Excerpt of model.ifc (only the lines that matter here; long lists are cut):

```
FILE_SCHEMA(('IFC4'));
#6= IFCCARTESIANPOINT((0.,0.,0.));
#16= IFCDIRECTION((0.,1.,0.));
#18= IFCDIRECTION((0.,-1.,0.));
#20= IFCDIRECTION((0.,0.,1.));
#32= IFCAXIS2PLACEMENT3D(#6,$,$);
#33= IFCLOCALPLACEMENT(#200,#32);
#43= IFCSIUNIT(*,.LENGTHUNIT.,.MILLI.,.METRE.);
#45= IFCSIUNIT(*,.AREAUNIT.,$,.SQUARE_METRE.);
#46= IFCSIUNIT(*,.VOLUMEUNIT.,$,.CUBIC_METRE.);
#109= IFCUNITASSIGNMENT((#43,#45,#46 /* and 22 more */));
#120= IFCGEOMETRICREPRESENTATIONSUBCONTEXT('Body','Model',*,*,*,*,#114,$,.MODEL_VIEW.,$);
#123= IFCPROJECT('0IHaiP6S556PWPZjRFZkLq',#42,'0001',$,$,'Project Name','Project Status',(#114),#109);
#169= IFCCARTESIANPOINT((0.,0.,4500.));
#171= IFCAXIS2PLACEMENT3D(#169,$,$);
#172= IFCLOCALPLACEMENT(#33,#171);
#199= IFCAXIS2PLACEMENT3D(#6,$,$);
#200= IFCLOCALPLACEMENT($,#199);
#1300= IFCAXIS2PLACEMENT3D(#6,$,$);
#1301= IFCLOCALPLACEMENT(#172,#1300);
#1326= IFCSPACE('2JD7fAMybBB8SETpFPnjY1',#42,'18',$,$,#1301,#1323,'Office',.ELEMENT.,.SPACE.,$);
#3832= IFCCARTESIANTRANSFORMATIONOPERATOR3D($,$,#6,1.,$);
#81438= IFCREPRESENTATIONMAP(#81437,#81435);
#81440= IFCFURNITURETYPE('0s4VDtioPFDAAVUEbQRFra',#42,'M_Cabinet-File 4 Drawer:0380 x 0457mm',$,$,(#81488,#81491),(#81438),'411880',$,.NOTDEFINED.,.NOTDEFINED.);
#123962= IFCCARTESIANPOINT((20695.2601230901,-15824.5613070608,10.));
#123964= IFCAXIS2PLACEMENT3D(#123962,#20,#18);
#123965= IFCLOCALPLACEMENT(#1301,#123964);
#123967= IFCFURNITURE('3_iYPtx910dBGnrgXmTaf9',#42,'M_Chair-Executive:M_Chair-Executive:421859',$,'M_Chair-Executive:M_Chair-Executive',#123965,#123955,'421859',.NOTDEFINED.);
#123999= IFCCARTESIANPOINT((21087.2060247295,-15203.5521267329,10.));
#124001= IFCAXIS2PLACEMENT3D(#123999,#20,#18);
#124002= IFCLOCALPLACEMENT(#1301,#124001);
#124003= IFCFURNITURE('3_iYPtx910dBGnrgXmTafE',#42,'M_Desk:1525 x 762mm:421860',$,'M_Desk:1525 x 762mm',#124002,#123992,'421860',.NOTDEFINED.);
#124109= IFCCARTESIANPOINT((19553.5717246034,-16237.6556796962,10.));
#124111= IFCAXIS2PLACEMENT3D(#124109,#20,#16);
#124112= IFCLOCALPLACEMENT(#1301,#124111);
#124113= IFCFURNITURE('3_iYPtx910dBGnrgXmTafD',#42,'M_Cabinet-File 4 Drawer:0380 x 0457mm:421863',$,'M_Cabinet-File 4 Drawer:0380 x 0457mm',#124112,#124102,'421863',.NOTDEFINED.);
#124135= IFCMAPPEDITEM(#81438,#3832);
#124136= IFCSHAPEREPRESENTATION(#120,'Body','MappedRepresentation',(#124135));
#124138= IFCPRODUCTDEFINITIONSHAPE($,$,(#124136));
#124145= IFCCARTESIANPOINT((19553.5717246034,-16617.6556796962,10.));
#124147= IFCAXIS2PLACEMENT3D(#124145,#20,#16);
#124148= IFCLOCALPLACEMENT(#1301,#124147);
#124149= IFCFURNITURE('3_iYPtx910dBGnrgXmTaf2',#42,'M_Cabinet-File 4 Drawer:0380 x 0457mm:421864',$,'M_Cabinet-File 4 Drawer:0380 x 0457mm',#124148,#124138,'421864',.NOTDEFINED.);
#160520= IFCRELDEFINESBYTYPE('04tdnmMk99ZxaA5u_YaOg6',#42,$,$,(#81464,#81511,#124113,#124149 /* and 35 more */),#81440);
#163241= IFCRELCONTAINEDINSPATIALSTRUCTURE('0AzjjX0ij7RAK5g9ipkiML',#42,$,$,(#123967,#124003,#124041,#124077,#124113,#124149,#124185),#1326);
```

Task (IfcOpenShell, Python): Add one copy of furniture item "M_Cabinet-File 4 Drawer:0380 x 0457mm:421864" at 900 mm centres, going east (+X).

```python
import numpy as np
import ifcopenshell
import ifcopenshell.api.geometry
import ifcopenshell.api.root
import ifcopenshell.util.element
import ifcopenshell.util.placement
import ifcopenshell.util.unit

model = ifcopenshell.open("model.ifc")
unit_scale = ifcopenshell.util.unit.calculate_unit_scale(model)


def reuse_history(source, copy):
    """copy_class also copies each property set's owner history, people and application; keep the originals."""
    for rel in copy.IsDefinedBy:
        if rel.is_a("IfcRelDefinesByProperties") and (history := rel.RelatingPropertyDefinition.OwnerHistory):
            rel.RelatingPropertyDefinition.OwnerHistory = source.OwnerHistory
            ifcopenshell.util.element.remove_deep2(model, history)


source = model.by_guid("3_iYPtx910dBGnrgXmTaf2")
base = ifcopenshell.util.placement.get_local_placement(source.ObjectPlacement)
step = np.array([1.0, 0.0, 0.0]) * 0.9 / unit_scale

for i in range(1, 2):
    copy = ifcopenshell.api.root.copy_class(model, product=source)
    copy.Representation = ifcopenshell.util.element.copy_deep(
        model, source.Representation, exclude=["IfcGeometricRepresentationContext", "IfcRepresentationMap"]
    )
    copy.Name = "M_Cabinet-File 4 Drawer:0380 x 0457mm"
    copy.Tag = None
    reuse_history(source, copy)
    matrix = base.copy()
    matrix[:3, 3] += i * step
    print("added at", matrix[:3, 3].round(3) + 0.0)
    ifcopenshell.api.geometry.edit_object_placement(model, product=copy, matrix=matrix, is_si=False)

model.write("model_edited.ifc")
```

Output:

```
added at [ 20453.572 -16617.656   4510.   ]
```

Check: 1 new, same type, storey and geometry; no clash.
